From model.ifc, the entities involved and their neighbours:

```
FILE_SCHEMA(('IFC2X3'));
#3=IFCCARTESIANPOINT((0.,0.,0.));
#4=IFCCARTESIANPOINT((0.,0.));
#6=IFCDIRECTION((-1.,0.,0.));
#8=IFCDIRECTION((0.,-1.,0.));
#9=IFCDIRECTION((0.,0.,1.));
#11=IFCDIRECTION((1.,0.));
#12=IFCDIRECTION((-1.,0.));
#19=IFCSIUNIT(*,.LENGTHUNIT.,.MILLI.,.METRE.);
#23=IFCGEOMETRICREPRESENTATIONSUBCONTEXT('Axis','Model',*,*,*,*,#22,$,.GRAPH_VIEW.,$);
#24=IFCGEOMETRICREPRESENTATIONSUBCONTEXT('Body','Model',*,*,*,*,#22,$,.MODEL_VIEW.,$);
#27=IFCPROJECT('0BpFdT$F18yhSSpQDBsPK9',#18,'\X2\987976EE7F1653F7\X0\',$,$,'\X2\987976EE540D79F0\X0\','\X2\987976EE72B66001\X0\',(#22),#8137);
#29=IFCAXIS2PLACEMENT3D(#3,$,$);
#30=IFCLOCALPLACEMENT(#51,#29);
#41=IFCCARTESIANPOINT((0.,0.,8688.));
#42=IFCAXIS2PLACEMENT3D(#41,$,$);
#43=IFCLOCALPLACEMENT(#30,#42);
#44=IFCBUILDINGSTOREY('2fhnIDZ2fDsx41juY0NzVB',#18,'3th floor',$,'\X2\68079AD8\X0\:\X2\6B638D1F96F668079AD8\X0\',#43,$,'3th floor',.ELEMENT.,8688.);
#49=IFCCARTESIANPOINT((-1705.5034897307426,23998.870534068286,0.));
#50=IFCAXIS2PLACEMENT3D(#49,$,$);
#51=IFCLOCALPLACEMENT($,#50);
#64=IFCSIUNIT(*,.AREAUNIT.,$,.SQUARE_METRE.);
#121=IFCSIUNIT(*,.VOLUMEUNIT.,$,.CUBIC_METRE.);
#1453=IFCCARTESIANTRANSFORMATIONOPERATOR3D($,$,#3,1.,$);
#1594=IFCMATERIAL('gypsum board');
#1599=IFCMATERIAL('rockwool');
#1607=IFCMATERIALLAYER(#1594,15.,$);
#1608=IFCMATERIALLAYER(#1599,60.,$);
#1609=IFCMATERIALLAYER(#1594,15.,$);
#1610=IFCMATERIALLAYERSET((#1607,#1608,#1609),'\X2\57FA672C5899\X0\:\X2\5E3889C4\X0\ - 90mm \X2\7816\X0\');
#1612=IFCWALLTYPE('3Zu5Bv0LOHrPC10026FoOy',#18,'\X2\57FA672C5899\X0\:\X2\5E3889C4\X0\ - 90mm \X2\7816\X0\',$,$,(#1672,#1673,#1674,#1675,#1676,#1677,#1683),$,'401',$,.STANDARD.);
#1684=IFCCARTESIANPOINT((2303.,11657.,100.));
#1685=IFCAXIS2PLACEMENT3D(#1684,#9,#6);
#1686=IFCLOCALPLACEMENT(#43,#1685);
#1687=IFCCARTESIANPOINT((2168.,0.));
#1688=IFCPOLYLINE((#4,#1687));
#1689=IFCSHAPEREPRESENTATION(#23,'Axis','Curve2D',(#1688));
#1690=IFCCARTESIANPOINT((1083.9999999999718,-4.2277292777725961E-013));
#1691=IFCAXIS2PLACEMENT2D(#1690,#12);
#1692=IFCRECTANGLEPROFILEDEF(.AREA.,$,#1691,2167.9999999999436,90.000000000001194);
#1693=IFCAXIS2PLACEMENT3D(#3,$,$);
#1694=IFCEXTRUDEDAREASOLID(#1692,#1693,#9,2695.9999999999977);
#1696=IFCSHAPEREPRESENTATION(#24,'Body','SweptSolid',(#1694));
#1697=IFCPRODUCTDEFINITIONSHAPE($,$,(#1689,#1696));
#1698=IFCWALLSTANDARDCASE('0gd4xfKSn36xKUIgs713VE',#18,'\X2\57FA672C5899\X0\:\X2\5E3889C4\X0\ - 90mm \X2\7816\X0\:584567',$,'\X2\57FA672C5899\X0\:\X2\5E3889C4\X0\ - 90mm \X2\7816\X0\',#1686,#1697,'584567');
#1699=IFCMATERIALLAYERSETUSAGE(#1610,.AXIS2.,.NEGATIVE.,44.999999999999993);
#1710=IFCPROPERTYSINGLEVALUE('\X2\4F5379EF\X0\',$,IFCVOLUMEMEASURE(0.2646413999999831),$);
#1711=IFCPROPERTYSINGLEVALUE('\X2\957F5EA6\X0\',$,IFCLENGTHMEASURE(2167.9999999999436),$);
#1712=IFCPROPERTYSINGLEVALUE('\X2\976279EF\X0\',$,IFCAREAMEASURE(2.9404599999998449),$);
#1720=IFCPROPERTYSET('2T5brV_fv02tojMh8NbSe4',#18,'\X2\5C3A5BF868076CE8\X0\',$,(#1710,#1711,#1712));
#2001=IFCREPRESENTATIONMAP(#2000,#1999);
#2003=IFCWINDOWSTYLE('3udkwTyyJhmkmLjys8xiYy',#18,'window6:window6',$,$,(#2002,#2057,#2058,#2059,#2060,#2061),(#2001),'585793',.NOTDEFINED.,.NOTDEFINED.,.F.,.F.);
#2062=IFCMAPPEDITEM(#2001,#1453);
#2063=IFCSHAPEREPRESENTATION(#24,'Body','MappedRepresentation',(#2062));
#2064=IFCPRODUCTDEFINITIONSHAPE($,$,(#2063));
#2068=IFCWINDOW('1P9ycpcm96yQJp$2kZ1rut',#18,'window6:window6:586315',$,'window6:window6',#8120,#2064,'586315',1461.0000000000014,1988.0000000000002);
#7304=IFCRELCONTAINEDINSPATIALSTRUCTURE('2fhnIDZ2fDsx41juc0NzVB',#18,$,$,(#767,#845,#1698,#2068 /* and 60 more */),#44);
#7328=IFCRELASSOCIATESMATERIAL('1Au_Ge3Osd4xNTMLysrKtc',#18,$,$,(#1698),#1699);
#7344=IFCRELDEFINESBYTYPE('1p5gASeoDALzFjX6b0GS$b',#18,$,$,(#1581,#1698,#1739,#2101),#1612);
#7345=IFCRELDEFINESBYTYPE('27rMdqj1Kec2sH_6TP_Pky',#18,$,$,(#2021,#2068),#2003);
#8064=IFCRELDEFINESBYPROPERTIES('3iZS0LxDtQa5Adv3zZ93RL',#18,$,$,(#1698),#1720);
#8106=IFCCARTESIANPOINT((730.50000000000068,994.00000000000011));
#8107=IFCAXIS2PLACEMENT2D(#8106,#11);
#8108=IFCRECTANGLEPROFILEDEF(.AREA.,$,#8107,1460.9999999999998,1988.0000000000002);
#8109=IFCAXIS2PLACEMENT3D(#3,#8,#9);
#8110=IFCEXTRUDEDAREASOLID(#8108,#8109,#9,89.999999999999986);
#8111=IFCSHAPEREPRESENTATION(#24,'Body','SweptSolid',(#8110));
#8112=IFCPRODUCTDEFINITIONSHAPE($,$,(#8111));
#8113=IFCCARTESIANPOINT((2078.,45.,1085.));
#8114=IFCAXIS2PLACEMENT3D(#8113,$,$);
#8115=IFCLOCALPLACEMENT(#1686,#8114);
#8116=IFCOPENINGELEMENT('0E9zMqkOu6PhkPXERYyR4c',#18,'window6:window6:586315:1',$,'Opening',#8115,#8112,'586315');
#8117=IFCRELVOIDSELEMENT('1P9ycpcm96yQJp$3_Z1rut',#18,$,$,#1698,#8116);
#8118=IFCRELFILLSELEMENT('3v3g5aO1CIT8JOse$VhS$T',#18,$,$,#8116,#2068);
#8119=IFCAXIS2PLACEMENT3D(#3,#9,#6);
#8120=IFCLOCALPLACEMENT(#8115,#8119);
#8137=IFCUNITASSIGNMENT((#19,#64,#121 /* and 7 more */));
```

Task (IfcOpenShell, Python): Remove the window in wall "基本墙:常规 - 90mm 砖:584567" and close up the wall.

```python
import ifcopenshell
import ifcopenshell.api.feature
import ifcopenshell.api.pset
import ifcopenshell.api.root
import ifcopenshell.geom
import ifcopenshell.util.element
import ifcopenshell.util.shape
import ifcopenshell.util.unit

model = ifcopenshell.open("model.ifc")
area_scale = ifcopenshell.util.unit.calculate_unit_scale(model, "AREAUNIT")
volume_scale = ifcopenshell.util.unit.calculate_unit_scale(model, "VOLUMEUNIT")
settings = ifcopenshell.geom.settings()


def volume(element):
    """Net volume in cubic metres, openings subtracted."""
    shape = ifcopenshell.geom.create_shape(settings, element)
    return ifcopenshell.util.shape.get_volume(shape.geometry)


window = model.by_id(2068)
opening = window.FillsVoids[0].RelatingOpeningElement
wall = opening.VoidsElements[0].RelatingBuildingElement
before = volume(wall)

ifcopenshell.api.root.remove_product(model, product=window)
ifcopenshell.api.feature.remove_feature(model, feature=opening)

after = volume(wall)
thickness = 0.09  # wall thickness in metres

# Update the wall's stored quantities.
pset = model.by_id(ifcopenshell.util.element.get_pset(wall, "尺寸标注", should_inherit=False)["id"])
ifcopenshell.api.pset.edit_pset(model, pset=pset, properties={
    "体积": model.create_entity("IfcVolumeMeasure", after / volume_scale),
    "面积": model.create_entity("IfcAreaMeasure", after / thickness / area_scale),
})

print(f"wall volume {before:.3f} -> {after:.3f} m3")

model.write("model_rev.ifc")
```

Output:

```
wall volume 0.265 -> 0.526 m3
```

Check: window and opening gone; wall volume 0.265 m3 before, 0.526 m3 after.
